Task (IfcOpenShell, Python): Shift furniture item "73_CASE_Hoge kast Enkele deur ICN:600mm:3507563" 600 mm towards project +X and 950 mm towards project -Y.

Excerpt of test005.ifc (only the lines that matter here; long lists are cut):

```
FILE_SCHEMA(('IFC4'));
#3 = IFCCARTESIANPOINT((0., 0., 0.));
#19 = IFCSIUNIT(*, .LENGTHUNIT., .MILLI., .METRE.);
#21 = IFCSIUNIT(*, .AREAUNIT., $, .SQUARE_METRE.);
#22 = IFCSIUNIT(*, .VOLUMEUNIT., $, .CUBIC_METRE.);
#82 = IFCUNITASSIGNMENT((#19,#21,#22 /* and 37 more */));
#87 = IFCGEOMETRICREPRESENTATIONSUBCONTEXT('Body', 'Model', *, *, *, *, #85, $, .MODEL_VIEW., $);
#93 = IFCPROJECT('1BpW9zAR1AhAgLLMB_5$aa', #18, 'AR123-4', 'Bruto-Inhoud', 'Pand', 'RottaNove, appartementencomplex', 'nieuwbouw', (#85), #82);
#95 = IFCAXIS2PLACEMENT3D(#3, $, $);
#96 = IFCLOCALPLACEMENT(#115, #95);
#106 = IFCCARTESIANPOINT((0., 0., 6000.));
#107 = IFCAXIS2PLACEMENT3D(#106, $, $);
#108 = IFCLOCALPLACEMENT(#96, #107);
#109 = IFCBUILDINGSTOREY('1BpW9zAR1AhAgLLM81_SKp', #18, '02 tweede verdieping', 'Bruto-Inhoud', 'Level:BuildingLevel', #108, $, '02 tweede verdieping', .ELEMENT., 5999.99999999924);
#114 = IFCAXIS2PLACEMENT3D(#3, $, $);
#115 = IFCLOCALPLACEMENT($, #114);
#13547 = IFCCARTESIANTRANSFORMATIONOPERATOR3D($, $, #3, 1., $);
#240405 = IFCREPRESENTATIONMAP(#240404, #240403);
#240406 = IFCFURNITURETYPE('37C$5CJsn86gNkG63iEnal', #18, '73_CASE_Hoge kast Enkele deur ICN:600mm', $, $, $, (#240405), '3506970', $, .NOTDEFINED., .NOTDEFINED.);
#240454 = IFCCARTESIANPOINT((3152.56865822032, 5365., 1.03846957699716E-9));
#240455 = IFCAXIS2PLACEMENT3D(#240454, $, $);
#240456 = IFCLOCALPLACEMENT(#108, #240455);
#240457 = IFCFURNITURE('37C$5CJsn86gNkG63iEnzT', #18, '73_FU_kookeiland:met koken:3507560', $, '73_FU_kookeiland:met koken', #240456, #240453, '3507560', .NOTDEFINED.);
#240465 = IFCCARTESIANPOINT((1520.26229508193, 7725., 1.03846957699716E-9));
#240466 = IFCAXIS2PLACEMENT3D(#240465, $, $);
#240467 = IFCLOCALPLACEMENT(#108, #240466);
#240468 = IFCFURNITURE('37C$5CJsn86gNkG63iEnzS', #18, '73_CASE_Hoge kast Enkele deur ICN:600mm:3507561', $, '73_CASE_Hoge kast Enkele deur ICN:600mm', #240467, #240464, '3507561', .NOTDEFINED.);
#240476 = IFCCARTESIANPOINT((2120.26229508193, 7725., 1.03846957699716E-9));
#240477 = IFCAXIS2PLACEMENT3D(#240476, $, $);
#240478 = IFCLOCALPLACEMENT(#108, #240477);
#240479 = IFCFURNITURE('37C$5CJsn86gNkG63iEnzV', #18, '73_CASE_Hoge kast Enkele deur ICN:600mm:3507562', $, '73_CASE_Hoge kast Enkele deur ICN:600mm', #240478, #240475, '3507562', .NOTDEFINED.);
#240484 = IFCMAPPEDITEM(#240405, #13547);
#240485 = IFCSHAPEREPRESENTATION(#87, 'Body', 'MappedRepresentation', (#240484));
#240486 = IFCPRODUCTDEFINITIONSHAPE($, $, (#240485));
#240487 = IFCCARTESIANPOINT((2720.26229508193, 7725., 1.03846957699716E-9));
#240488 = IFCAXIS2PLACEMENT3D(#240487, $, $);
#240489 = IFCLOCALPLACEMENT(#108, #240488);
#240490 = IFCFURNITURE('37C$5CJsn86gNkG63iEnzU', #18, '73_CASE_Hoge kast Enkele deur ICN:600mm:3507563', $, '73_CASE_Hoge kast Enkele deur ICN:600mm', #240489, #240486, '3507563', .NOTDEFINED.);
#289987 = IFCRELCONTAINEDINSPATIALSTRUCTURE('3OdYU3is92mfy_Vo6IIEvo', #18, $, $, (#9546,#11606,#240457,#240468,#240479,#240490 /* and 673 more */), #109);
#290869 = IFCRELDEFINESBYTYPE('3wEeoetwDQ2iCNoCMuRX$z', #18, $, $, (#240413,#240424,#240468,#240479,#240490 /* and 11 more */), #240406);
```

```python
import ifcopenshell
import ifcopenshell.api.geometry
import ifcopenshell.util.placement
import ifcopenshell.util.unit

model = ifcopenshell.open("test005.ifc")
unit_scale = ifcopenshell.util.unit.calculate_unit_scale(model)

item = model.by_guid("37C$5CJsn86gNkG63iEnzU")
matrix = ifcopenshell.util.placement.get_local_placement(item.ObjectPlacement)
matrix[0, 3] += 0.6 / unit_scale
matrix[1, 3] -= 0.95 / unit_scale
ifcopenshell.api.geometry.edit_object_placement(model, product=item, matrix=matrix, is_si=False)

print(ifcopenshell.util.placement.get_local_placement(item.ObjectPlacement).round(3) + 0.0)

model.write("test005-out.ifc")
```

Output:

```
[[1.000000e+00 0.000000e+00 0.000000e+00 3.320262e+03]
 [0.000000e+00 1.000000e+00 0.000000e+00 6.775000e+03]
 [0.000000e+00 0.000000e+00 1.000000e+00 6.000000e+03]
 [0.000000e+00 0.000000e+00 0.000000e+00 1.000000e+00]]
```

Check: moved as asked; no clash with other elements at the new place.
